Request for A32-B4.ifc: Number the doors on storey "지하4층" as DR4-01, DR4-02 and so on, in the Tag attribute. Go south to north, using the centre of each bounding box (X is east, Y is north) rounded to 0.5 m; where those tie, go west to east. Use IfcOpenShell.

First a look at what the model holds.

```python
import ifcopenshell
import ifcopenshell.util.element
import ifcopenshell.util.placement

model = ifcopenshell.open("A32-B4.ifc")
print(model.schema)
storey = next(s for s in model.by_type("IfcBuildingStorey") if s.Name == "지하4층")
doors = [e for e in ifcopenshell.util.element.get_decomposition(storey) if e.is_a("IfcDoor")]
for e in sorted(doors, key=lambda e: e.id()):
    origin = ifcopenshell.util.placement.get_local_placement(e.ObjectPlacement)[:3, 3]
    print(e.id(), e.Tag, e.Name, origin.round(2) + 0.0, sep=" | ")
```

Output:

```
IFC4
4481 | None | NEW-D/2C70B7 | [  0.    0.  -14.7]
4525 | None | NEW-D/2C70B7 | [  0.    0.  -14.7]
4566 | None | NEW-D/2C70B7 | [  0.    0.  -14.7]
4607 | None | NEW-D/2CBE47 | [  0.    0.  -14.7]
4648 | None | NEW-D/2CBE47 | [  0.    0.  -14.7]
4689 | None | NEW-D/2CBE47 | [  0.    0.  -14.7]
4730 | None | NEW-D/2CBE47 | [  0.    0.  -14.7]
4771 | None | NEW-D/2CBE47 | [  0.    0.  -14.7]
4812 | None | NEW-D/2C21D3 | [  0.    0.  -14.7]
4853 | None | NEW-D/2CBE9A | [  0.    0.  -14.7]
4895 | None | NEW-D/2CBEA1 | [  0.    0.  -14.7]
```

```python
import ifcopenshell
import ifcopenshell.geom
import ifcopenshell.util.element
import ifcopenshell.util.shape

model = ifcopenshell.open("A32-B4.ifc")
settings = ifcopenshell.geom.settings()
settings.set("use-world-coords", True)


def centre(element):
    shape = ifcopenshell.geom.create_shape(settings, element)
    return ifcopenshell.util.shape.get_bbox_centroid(shape.geometry)


storey = next(s for s in model.by_type("IfcBuildingStorey") if s.Name == "지하4층")
doors = [e for e in ifcopenshell.util.element.get_decomposition(storey) if e.is_a("IfcDoor")]

# Insertion points can sit at a corner or the storey origin, so sort by the geometry (in metres).
centres = {e: centre(e) for e in doors}
doors.sort(key=lambda e: (round(centres[e][1] / 0.5), centres[e][0]))

for i, e in enumerate(doors, start=1):
    number = f"DR4-{i:02d}"
    e.Tag = number
    print(e.id(), number)

model.write("A32-B4_updated.ifc")
```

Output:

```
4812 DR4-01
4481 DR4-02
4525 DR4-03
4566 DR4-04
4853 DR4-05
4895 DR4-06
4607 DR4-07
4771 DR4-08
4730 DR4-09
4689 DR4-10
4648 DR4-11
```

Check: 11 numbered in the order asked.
